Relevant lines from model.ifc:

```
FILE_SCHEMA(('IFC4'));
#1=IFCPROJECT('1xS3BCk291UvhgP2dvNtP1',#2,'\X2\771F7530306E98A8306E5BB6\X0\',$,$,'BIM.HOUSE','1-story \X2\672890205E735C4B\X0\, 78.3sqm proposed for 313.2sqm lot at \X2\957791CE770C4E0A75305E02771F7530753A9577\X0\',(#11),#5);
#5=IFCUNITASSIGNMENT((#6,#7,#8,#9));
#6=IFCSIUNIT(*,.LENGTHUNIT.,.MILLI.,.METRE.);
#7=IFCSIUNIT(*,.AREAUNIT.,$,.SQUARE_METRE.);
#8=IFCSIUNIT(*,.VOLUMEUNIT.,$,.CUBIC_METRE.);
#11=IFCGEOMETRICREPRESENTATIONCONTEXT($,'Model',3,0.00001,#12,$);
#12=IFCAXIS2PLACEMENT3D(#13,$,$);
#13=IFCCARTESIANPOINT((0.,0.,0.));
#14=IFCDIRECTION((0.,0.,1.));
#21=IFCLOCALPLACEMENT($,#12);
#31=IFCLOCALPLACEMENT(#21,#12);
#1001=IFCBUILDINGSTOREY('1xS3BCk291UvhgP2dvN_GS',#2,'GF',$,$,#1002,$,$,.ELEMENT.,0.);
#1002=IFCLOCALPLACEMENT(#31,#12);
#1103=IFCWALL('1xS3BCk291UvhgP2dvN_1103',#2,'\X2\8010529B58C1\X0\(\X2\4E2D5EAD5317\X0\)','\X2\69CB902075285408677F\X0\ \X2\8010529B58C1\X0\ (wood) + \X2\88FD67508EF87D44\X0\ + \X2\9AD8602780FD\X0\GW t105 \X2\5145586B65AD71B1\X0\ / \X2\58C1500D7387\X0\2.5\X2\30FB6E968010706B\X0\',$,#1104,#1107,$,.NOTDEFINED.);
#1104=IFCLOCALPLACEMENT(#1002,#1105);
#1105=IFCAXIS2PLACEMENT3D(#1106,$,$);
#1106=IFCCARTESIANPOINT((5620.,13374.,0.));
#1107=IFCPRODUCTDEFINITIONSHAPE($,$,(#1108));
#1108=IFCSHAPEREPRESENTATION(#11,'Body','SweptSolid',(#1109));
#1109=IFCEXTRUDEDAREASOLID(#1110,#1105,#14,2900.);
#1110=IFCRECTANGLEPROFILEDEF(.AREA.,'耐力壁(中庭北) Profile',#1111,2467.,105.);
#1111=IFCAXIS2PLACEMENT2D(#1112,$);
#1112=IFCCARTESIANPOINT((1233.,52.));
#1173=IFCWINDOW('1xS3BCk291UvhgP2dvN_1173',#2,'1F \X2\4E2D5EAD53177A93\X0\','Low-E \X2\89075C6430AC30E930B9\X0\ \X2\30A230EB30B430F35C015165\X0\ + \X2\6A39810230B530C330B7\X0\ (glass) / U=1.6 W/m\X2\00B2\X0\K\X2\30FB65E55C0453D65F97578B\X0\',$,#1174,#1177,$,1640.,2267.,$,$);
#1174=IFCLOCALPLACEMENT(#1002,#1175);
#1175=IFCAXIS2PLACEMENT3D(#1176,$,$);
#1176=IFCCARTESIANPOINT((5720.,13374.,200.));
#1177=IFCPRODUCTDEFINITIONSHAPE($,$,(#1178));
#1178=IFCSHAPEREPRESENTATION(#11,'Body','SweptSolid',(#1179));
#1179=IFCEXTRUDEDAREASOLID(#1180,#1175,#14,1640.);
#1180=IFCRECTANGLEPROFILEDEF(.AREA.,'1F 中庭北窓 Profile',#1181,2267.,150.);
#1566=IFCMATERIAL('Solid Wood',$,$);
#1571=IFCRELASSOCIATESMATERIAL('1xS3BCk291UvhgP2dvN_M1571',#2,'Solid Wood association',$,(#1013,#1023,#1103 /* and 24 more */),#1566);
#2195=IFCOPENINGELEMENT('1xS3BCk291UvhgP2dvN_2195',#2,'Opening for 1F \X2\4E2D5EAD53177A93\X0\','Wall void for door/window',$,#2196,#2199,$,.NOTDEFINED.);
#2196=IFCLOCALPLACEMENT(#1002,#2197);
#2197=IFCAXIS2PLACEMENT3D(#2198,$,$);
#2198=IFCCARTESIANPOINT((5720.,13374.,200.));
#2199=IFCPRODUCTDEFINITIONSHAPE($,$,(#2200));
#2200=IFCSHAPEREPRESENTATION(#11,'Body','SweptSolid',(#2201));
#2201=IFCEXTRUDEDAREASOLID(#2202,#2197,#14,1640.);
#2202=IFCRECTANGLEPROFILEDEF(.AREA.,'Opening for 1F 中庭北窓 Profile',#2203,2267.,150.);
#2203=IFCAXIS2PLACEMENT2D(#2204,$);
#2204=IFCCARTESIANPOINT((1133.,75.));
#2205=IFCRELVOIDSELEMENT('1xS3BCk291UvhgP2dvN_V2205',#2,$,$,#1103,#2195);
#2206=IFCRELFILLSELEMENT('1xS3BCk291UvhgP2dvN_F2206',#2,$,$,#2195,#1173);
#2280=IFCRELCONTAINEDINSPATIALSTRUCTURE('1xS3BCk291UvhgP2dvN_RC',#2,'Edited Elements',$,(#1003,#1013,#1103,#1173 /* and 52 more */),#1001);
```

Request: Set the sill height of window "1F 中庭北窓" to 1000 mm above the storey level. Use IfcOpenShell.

```python
import numpy as np
import ifcopenshell
import ifcopenshell.api.geometry
import ifcopenshell.geom
import ifcopenshell.util.element
import ifcopenshell.util.placement
import ifcopenshell.util.shape
import ifcopenshell.util.unit

model = ifcopenshell.open("model.ifc")
unit_scale = ifcopenshell.util.unit.calculate_unit_scale(model)

window = model.by_id(1173)
opening = window.FillsVoids[0].RelatingOpeningElement
storey = ifcopenshell.util.element.get_container(window, ifc_class="IfcBuildingStorey")
level = ifcopenshell.util.placement.get_local_placement(storey.ObjectPlacement)[2, 3]

# The opening's origin need not be at the sill, so measure its lowest point.
shape = ifcopenshell.geom.create_shape(ifcopenshell.geom.settings(), opening)
bottom = ifcopenshell.util.shape.get_shape_bottom_elevation(shape, shape.geometry) / unit_scale
dz = level + 1000.0 - bottom

shift = np.array([0.0, 0.0, dz])
# The window is not placed relative to its opening, so move both.
for product in (opening, window):
    matrix = ifcopenshell.util.placement.get_local_placement(product.ObjectPlacement)
    matrix[:3, 3] += shift
    ifcopenshell.api.geometry.edit_object_placement(model, product=product, matrix=matrix, is_si=False)

print(f"moved by {dz * unit_scale:+.3f} m")

model.write("model_edited.ifc")
```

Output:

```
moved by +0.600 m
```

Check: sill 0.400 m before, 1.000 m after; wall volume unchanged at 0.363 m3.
